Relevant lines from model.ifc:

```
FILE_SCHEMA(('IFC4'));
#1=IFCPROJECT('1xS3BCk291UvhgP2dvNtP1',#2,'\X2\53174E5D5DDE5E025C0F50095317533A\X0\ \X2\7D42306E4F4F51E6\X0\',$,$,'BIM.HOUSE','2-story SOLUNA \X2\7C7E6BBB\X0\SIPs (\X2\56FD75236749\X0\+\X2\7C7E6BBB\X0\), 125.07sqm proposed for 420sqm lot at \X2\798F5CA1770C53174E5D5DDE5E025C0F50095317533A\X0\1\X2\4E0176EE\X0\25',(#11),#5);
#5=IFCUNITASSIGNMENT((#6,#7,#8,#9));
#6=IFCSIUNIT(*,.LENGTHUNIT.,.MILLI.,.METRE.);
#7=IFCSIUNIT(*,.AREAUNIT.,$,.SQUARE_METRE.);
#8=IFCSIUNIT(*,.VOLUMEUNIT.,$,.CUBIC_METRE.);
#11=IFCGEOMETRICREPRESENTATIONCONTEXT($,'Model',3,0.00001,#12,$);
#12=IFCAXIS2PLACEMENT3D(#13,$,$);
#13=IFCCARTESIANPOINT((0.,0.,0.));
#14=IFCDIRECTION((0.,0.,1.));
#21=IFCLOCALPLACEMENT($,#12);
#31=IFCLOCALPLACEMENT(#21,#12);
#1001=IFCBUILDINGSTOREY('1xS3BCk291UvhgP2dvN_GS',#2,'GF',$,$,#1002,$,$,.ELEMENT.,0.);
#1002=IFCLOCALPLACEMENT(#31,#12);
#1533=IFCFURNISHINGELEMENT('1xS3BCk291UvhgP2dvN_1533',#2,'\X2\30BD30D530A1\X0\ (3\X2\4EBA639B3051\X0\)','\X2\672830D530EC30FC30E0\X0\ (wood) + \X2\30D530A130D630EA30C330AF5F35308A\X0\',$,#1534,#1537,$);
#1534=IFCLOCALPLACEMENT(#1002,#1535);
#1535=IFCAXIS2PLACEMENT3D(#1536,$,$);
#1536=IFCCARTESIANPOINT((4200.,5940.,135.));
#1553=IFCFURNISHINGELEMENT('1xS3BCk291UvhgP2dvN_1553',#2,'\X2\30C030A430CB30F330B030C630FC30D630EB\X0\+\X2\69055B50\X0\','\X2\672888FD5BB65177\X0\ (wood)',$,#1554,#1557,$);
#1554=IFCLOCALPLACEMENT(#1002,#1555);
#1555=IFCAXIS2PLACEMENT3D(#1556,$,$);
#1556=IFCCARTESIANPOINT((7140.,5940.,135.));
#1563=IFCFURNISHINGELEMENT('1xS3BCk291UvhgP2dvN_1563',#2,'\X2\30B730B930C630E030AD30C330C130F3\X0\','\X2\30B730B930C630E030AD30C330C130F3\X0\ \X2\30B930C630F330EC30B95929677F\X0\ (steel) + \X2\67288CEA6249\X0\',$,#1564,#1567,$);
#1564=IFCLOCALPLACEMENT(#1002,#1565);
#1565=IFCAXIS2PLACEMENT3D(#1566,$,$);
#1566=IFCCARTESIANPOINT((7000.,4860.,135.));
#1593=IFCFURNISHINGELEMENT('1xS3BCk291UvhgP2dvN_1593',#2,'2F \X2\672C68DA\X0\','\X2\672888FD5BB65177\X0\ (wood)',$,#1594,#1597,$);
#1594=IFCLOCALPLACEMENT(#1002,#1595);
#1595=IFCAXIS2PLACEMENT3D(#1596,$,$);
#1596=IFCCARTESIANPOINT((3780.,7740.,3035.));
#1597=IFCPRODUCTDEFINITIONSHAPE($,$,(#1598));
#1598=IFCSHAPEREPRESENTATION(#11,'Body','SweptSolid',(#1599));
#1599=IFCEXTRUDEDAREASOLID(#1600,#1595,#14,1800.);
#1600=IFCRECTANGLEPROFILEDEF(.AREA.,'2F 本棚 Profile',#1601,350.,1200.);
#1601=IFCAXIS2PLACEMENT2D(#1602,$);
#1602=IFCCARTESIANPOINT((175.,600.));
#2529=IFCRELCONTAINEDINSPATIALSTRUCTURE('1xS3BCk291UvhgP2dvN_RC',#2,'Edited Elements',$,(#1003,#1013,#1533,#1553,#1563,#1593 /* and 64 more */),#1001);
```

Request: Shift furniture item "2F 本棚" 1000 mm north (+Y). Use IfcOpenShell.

```python
import ifcopenshell
import ifcopenshell.api.geometry
import ifcopenshell.util.placement
import ifcopenshell.util.unit

model = ifcopenshell.open("model.ifc")
unit_scale = ifcopenshell.util.unit.calculate_unit_scale(model)

item = model.by_guid("1xS3BCk291UvhgP2dvN_1593")
matrix = ifcopenshell.util.placement.get_local_placement(item.ObjectPlacement)
matrix[1, 3] += 1 / unit_scale
ifcopenshell.api.geometry.edit_object_placement(model, product=item, matrix=matrix, is_si=False)

print(ifcopenshell.util.placement.get_local_placement(item.ObjectPlacement).round(3) + 0.0)

model.write("model_updated.ifc")
```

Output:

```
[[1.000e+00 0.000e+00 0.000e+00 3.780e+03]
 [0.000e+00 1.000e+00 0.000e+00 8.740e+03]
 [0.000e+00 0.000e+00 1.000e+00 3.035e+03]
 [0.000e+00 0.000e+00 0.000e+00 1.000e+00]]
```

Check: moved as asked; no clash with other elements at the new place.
